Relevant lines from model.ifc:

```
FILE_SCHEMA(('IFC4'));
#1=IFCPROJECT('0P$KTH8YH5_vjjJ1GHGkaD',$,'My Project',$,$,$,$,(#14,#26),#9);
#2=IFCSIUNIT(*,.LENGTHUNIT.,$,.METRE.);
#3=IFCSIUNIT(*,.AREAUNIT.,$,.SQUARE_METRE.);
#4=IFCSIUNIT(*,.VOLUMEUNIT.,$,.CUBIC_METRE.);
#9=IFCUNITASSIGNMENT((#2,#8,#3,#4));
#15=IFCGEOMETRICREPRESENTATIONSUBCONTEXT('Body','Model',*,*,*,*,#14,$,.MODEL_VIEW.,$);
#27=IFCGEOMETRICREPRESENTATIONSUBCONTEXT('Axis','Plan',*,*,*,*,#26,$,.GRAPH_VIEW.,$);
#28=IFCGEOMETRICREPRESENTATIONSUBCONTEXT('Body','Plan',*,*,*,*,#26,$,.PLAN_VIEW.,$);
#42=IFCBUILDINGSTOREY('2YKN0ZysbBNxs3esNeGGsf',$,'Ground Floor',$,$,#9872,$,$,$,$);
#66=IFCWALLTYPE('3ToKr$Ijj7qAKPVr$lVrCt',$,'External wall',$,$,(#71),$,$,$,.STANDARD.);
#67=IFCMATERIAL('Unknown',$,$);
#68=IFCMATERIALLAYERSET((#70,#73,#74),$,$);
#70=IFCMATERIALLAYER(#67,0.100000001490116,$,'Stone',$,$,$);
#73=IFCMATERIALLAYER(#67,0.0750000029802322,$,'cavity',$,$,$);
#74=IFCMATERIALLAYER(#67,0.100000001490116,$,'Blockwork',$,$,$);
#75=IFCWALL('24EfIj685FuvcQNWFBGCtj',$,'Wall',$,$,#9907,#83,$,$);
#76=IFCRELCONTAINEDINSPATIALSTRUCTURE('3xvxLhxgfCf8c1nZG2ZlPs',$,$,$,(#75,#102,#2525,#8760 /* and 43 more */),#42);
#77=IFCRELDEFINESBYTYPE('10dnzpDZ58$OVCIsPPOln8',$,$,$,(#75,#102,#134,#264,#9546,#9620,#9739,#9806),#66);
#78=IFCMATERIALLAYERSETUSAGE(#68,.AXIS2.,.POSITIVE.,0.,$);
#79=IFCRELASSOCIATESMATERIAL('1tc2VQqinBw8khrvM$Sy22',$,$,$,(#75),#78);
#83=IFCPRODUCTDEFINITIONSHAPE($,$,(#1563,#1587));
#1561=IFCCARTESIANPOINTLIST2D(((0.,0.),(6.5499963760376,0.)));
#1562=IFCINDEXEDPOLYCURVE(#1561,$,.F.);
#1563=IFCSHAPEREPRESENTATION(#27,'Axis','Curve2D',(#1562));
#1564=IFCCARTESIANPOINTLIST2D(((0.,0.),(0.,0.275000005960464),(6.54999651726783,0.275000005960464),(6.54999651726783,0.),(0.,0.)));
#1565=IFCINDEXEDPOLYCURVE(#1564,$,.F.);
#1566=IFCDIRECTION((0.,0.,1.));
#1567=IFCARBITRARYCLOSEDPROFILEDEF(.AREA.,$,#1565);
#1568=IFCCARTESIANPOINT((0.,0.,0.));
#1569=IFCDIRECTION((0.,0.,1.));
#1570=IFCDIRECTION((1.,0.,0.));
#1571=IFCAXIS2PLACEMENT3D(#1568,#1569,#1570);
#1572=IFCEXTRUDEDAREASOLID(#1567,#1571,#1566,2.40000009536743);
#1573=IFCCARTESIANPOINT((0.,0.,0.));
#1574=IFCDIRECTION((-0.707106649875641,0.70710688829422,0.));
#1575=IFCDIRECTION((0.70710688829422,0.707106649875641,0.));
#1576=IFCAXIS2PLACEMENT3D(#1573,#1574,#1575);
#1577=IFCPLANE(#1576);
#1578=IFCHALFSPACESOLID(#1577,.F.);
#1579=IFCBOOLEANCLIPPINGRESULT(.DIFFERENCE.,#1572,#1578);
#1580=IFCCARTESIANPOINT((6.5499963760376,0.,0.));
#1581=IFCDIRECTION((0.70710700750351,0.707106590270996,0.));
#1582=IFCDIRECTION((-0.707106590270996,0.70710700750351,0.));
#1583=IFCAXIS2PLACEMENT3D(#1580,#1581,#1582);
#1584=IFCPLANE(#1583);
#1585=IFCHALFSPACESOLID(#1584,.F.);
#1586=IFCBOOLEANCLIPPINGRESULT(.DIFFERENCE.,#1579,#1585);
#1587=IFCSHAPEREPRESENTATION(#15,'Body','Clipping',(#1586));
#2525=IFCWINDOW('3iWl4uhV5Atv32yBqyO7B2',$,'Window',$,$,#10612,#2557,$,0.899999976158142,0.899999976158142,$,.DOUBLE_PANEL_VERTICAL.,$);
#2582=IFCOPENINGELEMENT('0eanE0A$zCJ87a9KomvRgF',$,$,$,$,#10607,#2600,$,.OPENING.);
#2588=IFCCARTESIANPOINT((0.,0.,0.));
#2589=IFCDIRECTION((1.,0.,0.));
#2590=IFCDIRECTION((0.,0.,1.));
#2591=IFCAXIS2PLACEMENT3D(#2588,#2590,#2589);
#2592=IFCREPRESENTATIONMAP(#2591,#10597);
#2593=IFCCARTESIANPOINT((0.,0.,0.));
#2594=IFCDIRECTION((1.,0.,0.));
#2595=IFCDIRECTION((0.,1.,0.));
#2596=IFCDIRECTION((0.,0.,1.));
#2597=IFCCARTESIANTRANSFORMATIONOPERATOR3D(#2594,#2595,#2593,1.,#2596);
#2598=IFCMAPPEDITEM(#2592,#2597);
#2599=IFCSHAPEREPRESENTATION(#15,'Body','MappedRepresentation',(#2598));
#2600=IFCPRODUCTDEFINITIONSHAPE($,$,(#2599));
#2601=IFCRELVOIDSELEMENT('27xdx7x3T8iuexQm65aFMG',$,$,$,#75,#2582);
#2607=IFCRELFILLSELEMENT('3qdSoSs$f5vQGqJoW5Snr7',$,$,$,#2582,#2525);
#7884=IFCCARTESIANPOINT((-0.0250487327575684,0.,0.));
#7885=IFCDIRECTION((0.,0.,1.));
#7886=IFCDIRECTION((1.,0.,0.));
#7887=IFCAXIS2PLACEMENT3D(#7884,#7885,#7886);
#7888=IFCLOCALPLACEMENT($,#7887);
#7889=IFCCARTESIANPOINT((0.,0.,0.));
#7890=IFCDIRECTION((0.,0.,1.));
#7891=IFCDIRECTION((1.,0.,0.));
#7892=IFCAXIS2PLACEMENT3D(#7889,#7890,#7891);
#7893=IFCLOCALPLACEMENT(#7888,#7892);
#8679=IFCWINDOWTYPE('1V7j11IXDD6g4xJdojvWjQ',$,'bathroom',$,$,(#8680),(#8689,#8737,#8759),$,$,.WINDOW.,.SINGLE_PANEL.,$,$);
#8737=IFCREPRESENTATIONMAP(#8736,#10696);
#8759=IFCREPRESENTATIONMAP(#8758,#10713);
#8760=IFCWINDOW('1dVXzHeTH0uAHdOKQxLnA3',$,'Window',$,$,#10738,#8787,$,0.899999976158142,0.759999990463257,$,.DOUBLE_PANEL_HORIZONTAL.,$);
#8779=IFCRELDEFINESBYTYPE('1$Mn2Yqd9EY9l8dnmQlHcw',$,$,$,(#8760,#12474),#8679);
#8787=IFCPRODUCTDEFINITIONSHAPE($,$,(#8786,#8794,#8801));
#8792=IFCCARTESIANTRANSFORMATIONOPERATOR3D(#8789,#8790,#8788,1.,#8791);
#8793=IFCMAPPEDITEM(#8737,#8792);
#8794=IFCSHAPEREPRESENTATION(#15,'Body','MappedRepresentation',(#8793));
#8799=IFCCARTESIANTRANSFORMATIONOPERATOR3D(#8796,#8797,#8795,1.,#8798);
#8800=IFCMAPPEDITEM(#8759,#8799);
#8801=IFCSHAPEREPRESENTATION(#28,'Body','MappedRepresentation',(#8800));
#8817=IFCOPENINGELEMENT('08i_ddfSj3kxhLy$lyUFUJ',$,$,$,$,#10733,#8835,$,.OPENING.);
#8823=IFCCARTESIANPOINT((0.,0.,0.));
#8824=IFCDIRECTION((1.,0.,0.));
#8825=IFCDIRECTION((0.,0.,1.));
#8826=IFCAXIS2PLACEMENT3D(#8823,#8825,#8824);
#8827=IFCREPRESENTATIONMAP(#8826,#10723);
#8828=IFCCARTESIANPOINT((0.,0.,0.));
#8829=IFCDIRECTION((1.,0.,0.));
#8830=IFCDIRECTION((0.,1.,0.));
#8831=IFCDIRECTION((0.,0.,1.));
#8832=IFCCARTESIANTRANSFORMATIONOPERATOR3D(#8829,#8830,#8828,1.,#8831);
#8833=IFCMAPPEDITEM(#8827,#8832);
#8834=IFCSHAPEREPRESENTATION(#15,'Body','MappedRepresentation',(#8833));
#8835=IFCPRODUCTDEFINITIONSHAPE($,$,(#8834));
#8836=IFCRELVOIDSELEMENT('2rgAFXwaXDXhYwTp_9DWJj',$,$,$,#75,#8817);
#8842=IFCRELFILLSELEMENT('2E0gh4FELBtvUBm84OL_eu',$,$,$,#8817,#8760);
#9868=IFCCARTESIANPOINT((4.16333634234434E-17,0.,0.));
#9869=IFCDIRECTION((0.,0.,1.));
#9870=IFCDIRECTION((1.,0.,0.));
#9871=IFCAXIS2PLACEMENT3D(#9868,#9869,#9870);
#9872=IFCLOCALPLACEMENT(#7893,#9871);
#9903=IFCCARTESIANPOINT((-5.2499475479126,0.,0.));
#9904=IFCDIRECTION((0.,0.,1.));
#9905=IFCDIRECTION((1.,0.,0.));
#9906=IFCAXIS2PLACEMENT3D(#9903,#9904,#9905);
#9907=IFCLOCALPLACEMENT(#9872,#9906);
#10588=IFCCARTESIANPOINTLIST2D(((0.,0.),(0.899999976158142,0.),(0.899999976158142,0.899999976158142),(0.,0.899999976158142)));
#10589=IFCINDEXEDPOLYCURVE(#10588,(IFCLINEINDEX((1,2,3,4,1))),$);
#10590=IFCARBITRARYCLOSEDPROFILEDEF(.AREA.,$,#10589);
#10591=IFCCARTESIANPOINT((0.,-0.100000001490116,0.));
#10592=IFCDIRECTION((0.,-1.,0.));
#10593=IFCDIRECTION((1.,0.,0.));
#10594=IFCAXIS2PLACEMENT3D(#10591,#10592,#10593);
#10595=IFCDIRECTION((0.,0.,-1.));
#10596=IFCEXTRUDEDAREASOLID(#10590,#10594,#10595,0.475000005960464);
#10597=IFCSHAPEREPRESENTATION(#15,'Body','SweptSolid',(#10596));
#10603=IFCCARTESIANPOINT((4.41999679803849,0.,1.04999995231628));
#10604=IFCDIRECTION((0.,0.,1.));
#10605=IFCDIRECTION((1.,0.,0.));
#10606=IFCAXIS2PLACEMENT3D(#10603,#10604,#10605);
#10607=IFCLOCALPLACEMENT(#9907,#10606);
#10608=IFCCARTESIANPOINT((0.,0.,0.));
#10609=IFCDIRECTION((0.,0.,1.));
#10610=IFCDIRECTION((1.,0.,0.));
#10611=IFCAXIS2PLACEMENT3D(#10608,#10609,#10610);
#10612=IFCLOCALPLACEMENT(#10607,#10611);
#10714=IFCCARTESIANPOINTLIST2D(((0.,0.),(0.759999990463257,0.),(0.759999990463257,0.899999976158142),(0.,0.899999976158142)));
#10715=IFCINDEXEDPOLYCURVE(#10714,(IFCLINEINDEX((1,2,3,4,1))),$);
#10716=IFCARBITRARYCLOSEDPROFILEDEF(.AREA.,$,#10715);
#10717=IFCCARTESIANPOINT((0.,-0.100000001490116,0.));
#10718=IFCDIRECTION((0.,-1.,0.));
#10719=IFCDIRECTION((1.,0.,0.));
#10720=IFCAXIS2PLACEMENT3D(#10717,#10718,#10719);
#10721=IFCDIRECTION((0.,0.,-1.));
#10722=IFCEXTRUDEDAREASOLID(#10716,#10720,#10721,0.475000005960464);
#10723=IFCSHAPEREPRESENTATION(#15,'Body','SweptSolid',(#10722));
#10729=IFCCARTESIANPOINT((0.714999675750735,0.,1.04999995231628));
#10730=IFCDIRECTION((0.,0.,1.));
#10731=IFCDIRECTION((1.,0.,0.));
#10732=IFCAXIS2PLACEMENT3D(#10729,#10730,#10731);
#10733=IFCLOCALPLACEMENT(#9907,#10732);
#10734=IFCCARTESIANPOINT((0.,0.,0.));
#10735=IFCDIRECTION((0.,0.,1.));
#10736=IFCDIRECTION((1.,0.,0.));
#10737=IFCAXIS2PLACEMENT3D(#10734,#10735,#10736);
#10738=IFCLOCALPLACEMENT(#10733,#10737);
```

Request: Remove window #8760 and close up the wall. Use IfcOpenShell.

```python
import ifcopenshell
import ifcopenshell.api.feature
import ifcopenshell.api.root
import ifcopenshell.geom
import ifcopenshell.util.shape

model = ifcopenshell.open("model.ifc")
settings = ifcopenshell.geom.settings()


def volume(element):
    """Net volume in cubic metres, openings subtracted."""
    shape = ifcopenshell.geom.create_shape(settings, element)
    return ifcopenshell.util.shape.get_volume(shape.geometry)


window = model.by_guid("1dVXzHeTH0uAHdOKQxLnA3")
opening = window.FillsVoids[0].RelatingOpeningElement
wall = opening.VoidsElements[0].RelatingBuildingElement
before = volume(wall)

ifcopenshell.api.root.remove_product(model, product=window)
ifcopenshell.api.feature.remove_feature(model, feature=opening)

after = volume(wall)

print(f"wall volume {before:.3f} -> {after:.3f} m3")

model.write("model-out.ifc")
```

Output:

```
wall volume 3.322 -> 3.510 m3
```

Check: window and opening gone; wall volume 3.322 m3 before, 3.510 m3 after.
